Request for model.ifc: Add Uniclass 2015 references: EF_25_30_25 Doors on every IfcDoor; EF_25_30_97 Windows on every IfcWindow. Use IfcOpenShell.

First a look at what the model holds.

```python
import ifcopenshell

model = ifcopenshell.open("model.ifc")
print(model.schema)
print("classifications:", [c.Name for c in model.by_type("IfcClassification")])
for ifc_class in ("IfcDoor", "IfcRoof", "IfcStair", "IfcWall", "IfcWindow"):
    print(ifc_class, len(model.by_type(ifc_class)))
```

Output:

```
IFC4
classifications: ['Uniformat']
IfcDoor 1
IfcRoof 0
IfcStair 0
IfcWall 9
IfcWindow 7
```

```python
import ifcopenshell
import ifcopenshell.api.classification

model = ifcopenshell.open("model.ifc")

system = ifcopenshell.api.classification.add_classification(model, classification="Uniclass 2015")

codes = {
    "IfcDoor": ("EF_25_30_25", "Doors"),
    "IfcWindow": ("EF_25_30_97", "Windows"),
}
for ifc_class, (code, name) in codes.items():
    products = model.by_type(ifc_class)
    ifcopenshell.api.classification.add_reference(
        model, products=products, classification=system, identification=code, name=name
    )
    print(code, len(products))

model.write("model_rev.ifc")
```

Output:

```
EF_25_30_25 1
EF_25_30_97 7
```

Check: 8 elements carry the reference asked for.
